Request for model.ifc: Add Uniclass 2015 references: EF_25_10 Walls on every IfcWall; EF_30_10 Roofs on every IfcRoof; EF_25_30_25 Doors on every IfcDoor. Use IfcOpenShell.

First a look at what the model holds.

```python
import ifcopenshell

model = ifcopenshell.open("model.ifc")
print(model.schema)
print("classifications:", [c.Name for c in model.by_type("IfcClassification")])
for ifc_class in ("IfcDoor", "IfcRoof", "IfcStair", "IfcWall", "IfcWindow"):
    print(ifc_class, len(model.by_type(ifc_class)))
```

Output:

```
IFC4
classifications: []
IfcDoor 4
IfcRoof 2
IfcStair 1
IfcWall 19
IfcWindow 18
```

```python
import ifcopenshell
import ifcopenshell.api.classification

model = ifcopenshell.open("model.ifc")

system = ifcopenshell.api.classification.add_classification(model, classification="Uniclass 2015")

codes = {
    "IfcWall": ("EF_25_10", "Walls"),
    "IfcRoof": ("EF_30_10", "Roofs"),
    "IfcDoor": ("EF_25_30_25", "Doors"),
}
for ifc_class, (code, name) in codes.items():
    products = model.by_type(ifc_class)
    ifcopenshell.api.classification.add_reference(
        model, products=products, classification=system, identification=code, name=name
    )
    print(code, len(products))

model.write("model_edited.ifc")
```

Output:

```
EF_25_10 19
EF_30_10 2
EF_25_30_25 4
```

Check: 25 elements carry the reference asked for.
